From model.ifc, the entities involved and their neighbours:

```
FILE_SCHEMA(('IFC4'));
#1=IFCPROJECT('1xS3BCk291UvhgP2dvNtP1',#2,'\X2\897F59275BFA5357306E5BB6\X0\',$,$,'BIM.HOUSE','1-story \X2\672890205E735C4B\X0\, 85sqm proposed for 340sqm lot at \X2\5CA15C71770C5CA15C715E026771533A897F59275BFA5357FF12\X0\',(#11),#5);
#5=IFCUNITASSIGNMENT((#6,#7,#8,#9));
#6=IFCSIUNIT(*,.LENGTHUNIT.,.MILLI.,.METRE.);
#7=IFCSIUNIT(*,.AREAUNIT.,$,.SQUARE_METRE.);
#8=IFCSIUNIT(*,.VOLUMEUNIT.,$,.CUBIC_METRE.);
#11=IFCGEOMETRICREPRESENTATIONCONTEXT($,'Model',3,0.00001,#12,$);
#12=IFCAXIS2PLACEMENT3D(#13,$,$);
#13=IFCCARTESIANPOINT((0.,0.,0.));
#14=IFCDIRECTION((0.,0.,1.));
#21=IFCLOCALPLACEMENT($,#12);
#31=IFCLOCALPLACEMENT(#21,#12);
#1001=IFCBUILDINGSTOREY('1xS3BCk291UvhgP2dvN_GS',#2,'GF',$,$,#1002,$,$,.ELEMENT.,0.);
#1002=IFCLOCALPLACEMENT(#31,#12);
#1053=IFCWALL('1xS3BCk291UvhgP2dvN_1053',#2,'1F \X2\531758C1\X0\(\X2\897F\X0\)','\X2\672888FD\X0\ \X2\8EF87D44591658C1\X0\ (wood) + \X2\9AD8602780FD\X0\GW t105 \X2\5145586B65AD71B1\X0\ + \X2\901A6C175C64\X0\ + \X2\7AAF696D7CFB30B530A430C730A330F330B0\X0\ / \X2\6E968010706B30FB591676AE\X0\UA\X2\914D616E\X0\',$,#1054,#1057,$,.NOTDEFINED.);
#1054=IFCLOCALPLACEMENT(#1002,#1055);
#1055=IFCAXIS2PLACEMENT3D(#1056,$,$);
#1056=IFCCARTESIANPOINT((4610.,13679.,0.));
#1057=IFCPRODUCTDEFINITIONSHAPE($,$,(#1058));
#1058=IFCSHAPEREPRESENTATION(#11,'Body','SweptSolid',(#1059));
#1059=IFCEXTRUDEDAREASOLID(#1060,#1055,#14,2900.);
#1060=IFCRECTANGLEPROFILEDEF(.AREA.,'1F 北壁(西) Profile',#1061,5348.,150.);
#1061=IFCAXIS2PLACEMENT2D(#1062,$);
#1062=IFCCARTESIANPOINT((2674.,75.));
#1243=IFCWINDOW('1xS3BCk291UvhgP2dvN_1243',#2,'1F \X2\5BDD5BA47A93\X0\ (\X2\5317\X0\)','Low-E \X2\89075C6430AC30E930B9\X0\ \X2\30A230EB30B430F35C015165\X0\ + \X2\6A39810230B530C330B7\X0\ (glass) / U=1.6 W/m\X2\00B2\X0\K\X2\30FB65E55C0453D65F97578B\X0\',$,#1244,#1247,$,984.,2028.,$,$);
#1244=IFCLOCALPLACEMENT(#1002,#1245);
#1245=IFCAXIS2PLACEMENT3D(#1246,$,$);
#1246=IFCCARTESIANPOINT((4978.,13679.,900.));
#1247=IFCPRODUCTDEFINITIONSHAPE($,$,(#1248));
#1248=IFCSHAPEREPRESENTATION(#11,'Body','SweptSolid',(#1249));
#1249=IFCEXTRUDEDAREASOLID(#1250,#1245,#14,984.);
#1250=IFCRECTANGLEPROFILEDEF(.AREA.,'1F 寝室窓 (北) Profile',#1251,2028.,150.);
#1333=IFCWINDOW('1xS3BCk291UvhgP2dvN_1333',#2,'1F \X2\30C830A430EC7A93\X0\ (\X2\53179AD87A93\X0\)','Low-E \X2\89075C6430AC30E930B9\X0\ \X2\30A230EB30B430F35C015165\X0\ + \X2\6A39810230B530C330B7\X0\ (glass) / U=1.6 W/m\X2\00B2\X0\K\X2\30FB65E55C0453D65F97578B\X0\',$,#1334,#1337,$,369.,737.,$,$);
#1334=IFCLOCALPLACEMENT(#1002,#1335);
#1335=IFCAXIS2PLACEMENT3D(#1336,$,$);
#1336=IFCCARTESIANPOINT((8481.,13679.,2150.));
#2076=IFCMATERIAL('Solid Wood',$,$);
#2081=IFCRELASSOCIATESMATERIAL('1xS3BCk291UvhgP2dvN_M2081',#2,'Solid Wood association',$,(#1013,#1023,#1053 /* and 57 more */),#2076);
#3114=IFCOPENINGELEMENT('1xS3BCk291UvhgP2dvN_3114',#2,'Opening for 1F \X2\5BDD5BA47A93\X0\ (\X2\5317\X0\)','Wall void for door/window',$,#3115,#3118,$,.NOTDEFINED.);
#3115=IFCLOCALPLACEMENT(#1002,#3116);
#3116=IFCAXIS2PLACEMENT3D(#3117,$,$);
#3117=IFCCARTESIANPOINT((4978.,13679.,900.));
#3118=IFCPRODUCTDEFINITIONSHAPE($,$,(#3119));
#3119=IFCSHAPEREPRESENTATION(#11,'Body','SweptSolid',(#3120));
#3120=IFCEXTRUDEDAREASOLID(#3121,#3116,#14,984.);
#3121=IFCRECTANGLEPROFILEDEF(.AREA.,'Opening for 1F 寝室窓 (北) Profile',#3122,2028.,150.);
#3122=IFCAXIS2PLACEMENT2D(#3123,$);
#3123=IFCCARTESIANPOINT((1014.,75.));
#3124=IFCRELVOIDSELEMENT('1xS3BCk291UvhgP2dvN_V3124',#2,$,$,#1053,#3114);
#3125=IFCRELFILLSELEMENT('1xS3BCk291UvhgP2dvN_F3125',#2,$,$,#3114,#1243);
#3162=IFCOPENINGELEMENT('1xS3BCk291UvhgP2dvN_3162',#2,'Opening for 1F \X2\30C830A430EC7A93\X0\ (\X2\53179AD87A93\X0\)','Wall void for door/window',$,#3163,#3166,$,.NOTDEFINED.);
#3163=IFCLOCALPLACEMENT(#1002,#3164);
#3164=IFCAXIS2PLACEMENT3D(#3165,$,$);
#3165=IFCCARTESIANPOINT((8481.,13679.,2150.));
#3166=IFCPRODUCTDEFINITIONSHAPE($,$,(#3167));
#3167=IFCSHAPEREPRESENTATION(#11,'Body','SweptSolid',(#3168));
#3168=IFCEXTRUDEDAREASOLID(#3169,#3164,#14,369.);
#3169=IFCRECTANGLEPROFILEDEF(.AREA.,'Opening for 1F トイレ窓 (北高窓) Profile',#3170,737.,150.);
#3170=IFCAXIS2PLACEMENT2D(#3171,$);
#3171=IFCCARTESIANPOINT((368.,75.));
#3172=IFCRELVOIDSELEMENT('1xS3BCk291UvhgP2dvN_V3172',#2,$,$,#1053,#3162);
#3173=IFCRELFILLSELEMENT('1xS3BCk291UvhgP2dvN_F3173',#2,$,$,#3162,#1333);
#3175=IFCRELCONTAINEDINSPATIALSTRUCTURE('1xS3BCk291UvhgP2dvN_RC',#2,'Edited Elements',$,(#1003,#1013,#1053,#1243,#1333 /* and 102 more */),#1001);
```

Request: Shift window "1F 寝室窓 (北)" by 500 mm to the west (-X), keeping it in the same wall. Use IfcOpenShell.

```python
import ifcopenshell
import ifcopenshell.api.geometry
import ifcopenshell.util.placement

model = ifcopenshell.open("model.ifc")

window = model.by_id(1243)
opening = window.FillsVoids[0].RelatingOpeningElement
wall = opening.VoidsElements[0].RelatingBuildingElement

wall_matrix = ifcopenshell.util.placement.get_local_placement(wall.ObjectPlacement)
shift = wall_matrix[:3, 0] * -500.0
before = ifcopenshell.util.placement.get_local_placement(window.ObjectPlacement)[:3, 3].copy()

# The window is not placed relative to its opening, so move both.
for product in (opening, window):
    matrix = ifcopenshell.util.placement.get_local_placement(product.ObjectPlacement)
    matrix[:3, 3] += shift
    ifcopenshell.api.geometry.edit_object_placement(model, product=product, matrix=matrix, is_si=False)

after = ifcopenshell.util.placement.get_local_placement(window.ObjectPlacement)[:3, 3]
print("window moved by", (after - before).round(3) + 0.0)

model.write("model-out.ifc")
```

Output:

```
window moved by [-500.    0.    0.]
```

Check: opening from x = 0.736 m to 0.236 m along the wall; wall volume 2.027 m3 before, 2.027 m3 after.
